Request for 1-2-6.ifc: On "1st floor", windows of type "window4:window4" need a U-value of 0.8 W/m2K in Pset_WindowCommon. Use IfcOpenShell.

First a look at what the model holds.

```python
import ifcopenshell
import ifcopenshell.util.element

model = ifcopenshell.open("1-2-6.ifc")
print(model.schema)
storey = next(s for s in model.by_type("IfcBuildingStorey") if s.Name == "1st floor")
windows = [e for e in ifcopenshell.util.element.get_decomposition(storey) if e.is_a("IfcWindow")]
seen = {}
for e in windows:
    element_type = ifcopenshell.util.element.get_type(e)
    key = (element_type.Name if element_type != e and element_type else None, ifcopenshell.util.element.get_pset(e, "Pset_WindowCommon", "ThermalTransmittance"))
    seen[key] = seen.get(key, 0) + 1
for (name, value), count in sorted(seen.items(), key=str):
    print(count, "x", name, "|", value)
```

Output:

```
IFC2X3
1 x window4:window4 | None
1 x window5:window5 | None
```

```python
import ifcopenshell
import ifcopenshell.api.pset
import ifcopenshell.util.element

model = ifcopenshell.open("1-2-6.ifc")

storey = next(s for s in model.by_type("IfcBuildingStorey") if s.Name == "1st floor")
windows = [e for e in ifcopenshell.util.element.get_decomposition(storey) if e.is_a("IfcWindow")]

count = 0
for e in windows:
    element_type = ifcopenshell.util.element.get_type(e)
    if element_type in (None, e) or element_type.Name != "window4:window4":
        continue
    # add_pset returns the element's existing set when there is one.
    pset = ifcopenshell.api.pset.add_pset(model, product=e, name="Pset_WindowCommon")
    ifcopenshell.api.pset.edit_pset(model, pset=pset, properties={"ThermalTransmittance": 0.8})
    count += 1

print(count, "windows updated")

model.write("1-2-6_updated.ifc")
```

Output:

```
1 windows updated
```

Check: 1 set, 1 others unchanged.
